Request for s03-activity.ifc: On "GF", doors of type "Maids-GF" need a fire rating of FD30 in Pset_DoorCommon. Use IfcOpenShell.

First a look at what the model holds.

```python
import ifcopenshell
import ifcopenshell.util.element

model = ifcopenshell.open("s03-activity.ifc")
print(model.schema)
storey = next(s for s in model.by_type("IfcBuildingStorey") if s.Name == "GF")
doors = [e for e in ifcopenshell.util.element.get_decomposition(storey) if e.is_a("IfcDoor")]
seen = {}
for e in doors:
    element_type = ifcopenshell.util.element.get_type(e)
    key = (element_type.Name if element_type != e and element_type else None, ifcopenshell.util.element.get_pset(e, "Pset_DoorCommon", "FireRating"))
    seen[key] = seen.get(key, 0) + 1
for (name, value), count in sorted(seen.items(), key=str):
    print(count, "x", name, "|", value)
```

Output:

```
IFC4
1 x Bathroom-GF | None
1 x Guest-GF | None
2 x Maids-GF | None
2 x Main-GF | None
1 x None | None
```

```python
import ifcopenshell
import ifcopenshell.api.pset
import ifcopenshell.util.element

model = ifcopenshell.open("s03-activity.ifc")

storey = next(s for s in model.by_type("IfcBuildingStorey") if s.Name == "GF")
doors = [e for e in ifcopenshell.util.element.get_decomposition(storey) if e.is_a("IfcDoor")]

count = 0
for e in doors:
    element_type = ifcopenshell.util.element.get_type(e)
    if element_type in (None, e) or element_type.Name != "Maids-GF":
        continue
    # add_pset returns the element's existing set when there is one.
    pset = ifcopenshell.api.pset.add_pset(model, product=e, name="Pset_DoorCommon")
    ifcopenshell.api.pset.edit_pset(model, pset=pset, properties={"FireRating": "FD30"})
    count += 1

print(count, "doors updated")

model.write("s03-activity_edited.ifc")
```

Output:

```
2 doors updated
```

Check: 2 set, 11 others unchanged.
